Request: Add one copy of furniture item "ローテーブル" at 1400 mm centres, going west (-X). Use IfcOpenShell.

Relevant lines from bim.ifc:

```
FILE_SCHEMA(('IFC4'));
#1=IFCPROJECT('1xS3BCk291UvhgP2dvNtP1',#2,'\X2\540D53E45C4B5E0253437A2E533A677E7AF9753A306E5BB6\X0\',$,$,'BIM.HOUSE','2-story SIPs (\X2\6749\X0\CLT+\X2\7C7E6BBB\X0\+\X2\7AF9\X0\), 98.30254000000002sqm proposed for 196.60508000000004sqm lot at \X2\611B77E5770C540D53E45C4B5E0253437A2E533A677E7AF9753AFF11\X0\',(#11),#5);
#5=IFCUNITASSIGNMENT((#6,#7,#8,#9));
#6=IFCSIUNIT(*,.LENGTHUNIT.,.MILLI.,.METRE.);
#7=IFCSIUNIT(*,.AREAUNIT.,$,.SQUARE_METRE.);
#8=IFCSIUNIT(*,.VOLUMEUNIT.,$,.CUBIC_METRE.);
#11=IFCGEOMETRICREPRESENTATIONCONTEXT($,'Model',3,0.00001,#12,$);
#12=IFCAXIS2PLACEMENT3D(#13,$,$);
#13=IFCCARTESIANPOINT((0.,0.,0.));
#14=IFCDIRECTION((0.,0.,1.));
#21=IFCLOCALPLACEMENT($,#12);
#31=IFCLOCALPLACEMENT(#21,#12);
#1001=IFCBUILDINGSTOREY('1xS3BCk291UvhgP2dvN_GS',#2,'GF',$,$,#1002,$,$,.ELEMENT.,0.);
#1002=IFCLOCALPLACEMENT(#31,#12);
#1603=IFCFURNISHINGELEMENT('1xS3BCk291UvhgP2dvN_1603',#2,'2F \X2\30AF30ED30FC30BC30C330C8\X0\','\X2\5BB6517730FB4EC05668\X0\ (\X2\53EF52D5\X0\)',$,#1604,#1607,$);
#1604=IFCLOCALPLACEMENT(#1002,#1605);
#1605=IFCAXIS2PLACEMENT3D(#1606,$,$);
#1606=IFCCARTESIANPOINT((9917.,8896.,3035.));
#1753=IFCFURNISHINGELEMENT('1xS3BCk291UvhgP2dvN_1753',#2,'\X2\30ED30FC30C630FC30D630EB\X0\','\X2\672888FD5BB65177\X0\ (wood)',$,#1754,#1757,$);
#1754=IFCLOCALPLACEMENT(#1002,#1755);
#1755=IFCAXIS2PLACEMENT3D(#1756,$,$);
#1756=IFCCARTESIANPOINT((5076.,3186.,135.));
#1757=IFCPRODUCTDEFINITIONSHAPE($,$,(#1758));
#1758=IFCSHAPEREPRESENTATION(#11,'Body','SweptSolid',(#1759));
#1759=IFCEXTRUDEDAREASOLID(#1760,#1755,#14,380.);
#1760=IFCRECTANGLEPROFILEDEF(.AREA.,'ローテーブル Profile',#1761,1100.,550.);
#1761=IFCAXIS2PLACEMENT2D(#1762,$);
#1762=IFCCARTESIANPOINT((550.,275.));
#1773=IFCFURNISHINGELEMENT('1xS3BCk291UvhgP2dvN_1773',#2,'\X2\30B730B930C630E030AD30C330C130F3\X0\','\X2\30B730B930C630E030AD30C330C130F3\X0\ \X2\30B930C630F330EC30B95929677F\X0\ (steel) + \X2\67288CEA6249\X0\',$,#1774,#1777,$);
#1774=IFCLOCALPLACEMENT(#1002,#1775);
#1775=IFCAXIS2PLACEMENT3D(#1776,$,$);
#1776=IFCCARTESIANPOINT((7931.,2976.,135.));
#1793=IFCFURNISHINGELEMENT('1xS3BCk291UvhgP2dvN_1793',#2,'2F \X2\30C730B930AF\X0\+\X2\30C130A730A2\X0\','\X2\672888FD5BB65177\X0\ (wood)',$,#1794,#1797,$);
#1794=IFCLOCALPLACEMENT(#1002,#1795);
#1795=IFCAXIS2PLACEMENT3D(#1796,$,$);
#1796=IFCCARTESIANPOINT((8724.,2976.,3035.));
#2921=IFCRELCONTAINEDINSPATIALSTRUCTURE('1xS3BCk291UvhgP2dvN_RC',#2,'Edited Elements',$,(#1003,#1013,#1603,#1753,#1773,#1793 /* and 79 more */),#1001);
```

```python
import numpy as np
import ifcopenshell
import ifcopenshell.api.geometry
import ifcopenshell.api.root
import ifcopenshell.util.element
import ifcopenshell.util.placement
import ifcopenshell.util.unit

model = ifcopenshell.open("bim.ifc")
unit_scale = ifcopenshell.util.unit.calculate_unit_scale(model)


def reuse_history(source, copy):
    """copy_class also copies each property set's owner history, people and application; keep the originals."""
    for rel in copy.IsDefinedBy:
        if rel.is_a("IfcRelDefinesByProperties") and (history := rel.RelatingPropertyDefinition.OwnerHistory):
            rel.RelatingPropertyDefinition.OwnerHistory = source.OwnerHistory
            ifcopenshell.util.element.remove_deep2(model, history)


source = model.by_id(1753)
base = ifcopenshell.util.placement.get_local_placement(source.ObjectPlacement)
step = np.array([-1.0, 0.0, 0.0]) * 1.4 / unit_scale

for i in range(1, 2):
    copy = ifcopenshell.api.root.copy_class(model, product=source)
    copy.Representation = ifcopenshell.util.element.copy_deep(
        model, source.Representation, exclude=["IfcGeometricRepresentationContext", "IfcRepresentationMap"]
    )
    reuse_history(source, copy)
    matrix = base.copy()
    matrix[:3, 3] += i * step
    print("added at", matrix[:3, 3].round(3) + 0.0)
    ifcopenshell.api.geometry.edit_object_placement(model, product=copy, matrix=matrix, is_si=False)

model.write("bim_v2.ifc")
```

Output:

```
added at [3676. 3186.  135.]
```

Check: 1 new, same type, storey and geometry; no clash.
